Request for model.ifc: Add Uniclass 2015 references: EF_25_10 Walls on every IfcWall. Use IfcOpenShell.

First a look at what the model holds.

```python
import ifcopenshell

model = ifcopenshell.open("model.ifc")
print(model.schema)
print("classifications:", [c.Name for c in model.by_type("IfcClassification")])
for ifc_class in ("IfcDoor", "IfcRoof", "IfcStair", "IfcWall", "IfcWindow"):
    print(ifc_class, len(model.by_type(ifc_class)))
```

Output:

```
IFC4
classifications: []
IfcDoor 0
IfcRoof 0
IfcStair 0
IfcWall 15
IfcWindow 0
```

```python
import ifcopenshell
import ifcopenshell.api.classification

model = ifcopenshell.open("model.ifc")

system = ifcopenshell.api.classification.add_classification(model, classification="Uniclass 2015")

codes = {
    "IfcWall": ("EF_25_10", "Walls"),
}
for ifc_class, (code, name) in codes.items():
    products = model.by_type(ifc_class)
    ifcopenshell.api.classification.add_reference(
        model, products=products, classification=system, identification=code, name=name
    )
    print(code, len(products))

model.write("model_rev.ifc")
```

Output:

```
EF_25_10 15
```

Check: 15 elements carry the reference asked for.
